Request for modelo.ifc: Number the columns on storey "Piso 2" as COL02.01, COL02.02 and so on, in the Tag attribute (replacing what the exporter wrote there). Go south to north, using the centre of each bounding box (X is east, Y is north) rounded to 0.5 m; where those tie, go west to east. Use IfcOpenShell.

First a look at what the model holds.

```python
import ifcopenshell
import ifcopenshell.util.element
import ifcopenshell.util.placement

model = ifcopenshell.open("modelo.ifc")
print(model.schema)
storey = next(s for s in model.by_type("IfcBuildingStorey") if s.Name == "Piso 2")
columns = [e for e in ifcopenshell.util.element.get_decomposition(storey) if e.is_a("IfcColumn")]
for e in sorted(columns, key=lambda e: e.id()):
    origin = ifcopenshell.util.placement.get_local_placement(e.ObjectPlacement)[:3, 3]
    print(e.id(), e.Tag, e.Name, origin.round(2) + 0.0, sep=" | ")
```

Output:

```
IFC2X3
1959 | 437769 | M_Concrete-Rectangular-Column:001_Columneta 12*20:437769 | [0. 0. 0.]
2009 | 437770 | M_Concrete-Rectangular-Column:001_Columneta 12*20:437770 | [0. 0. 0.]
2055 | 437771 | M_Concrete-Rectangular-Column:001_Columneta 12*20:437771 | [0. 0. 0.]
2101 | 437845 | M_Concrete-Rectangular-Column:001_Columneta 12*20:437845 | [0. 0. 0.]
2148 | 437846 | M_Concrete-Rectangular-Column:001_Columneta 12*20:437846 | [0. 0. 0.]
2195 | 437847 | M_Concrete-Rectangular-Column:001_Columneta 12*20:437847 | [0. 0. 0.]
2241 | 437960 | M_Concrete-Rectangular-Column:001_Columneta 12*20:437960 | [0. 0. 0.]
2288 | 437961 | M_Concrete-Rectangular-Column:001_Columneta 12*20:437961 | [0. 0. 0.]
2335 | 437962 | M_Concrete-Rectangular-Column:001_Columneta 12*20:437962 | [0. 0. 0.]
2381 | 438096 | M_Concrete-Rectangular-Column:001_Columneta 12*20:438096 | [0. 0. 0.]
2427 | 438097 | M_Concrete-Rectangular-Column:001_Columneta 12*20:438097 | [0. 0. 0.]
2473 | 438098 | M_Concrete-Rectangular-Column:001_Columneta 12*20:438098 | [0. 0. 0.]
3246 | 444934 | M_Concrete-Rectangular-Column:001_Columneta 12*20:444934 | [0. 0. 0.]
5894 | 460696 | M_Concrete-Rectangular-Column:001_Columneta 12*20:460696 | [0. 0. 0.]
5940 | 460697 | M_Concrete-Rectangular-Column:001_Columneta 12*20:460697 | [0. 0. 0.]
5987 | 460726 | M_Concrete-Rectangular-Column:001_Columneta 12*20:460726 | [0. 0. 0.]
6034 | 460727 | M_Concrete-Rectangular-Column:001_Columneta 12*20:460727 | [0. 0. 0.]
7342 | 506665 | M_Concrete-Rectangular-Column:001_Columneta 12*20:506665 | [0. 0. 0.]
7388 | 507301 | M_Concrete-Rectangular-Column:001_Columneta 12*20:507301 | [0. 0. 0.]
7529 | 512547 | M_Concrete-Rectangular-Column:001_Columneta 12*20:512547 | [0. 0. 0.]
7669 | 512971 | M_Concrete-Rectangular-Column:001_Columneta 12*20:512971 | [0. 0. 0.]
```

```python
import ifcopenshell
import ifcopenshell.geom
import ifcopenshell.util.element
import ifcopenshell.util.shape

model = ifcopenshell.open("modelo.ifc")
settings = ifcopenshell.geom.settings()
settings.set("use-world-coords", True)


def centre(element):
    shape = ifcopenshell.geom.create_shape(settings, element)
    return ifcopenshell.util.shape.get_bbox_centroid(shape.geometry)


storey = next(s for s in model.by_type("IfcBuildingStorey") if s.Name == "Piso 2")
columns = [e for e in ifcopenshell.util.element.get_decomposition(storey) if e.is_a("IfcColumn")]

# Insertion points can sit at a corner or the storey origin, so sort by the geometry (in metres).
centres = {e: centre(e) for e in columns}
columns.sort(key=lambda e: (round(centres[e][1] / 0.5), centres[e][0]))

for i, e in enumerate(columns, start=1):
    number = f"COL02.{i:02d}"
    e.Tag = number
    print(e.id(), number)

model.write("modelo_edited.ifc")
```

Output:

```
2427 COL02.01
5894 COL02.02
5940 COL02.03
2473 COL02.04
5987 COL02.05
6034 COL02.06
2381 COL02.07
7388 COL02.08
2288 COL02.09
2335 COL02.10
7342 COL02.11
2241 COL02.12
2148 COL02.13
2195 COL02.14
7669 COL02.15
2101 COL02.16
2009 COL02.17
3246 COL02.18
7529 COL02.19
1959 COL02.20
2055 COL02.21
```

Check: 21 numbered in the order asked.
